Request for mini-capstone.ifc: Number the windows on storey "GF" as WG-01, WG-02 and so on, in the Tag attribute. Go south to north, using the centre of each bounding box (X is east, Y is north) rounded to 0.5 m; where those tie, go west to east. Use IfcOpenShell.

First a look at what the model holds.

```python
import ifcopenshell
import ifcopenshell.util.element
import ifcopenshell.util.placement

model = ifcopenshell.open("mini-capstone.ifc")
print(model.schema)
storey = next(s for s in model.by_type("IfcBuildingStorey") if s.Name == "GF")
windows = [e for e in ifcopenshell.util.element.get_decomposition(storey) if e.is_a("IfcWindow")]
for e in sorted(windows, key=lambda e: e.id()):
    origin = ifcopenshell.util.placement.get_local_placement(e.ObjectPlacement)[:3, 3]
    print(e.id(), e.Tag, e.Name, origin.round(2) + 0.0, sep=" | ")
```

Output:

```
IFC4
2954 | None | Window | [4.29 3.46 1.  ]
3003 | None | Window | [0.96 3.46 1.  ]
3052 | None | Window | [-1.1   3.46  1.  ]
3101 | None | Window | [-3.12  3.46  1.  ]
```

```python
import ifcopenshell
import ifcopenshell.geom
import ifcopenshell.util.element
import ifcopenshell.util.shape

model = ifcopenshell.open("mini-capstone.ifc")
settings = ifcopenshell.geom.settings()
settings.set("use-world-coords", True)


def centre(element):
    shape = ifcopenshell.geom.create_shape(settings, element)
    return ifcopenshell.util.shape.get_bbox_centroid(shape.geometry)


storey = next(s for s in model.by_type("IfcBuildingStorey") if s.Name == "GF")
windows = [e for e in ifcopenshell.util.element.get_decomposition(storey) if e.is_a("IfcWindow")]

# Insertion points can sit at a corner or the storey origin, so sort by the geometry (in metres).
centres = {e: centre(e) for e in windows}
windows.sort(key=lambda e: (round(centres[e][1] / 0.5), centres[e][0]))

for i, e in enumerate(windows, start=1):
    number = f"WG-{i:02d}"
    e.Tag = number
    print(e.id(), number)

model.write("mini-capstone_edited.ifc")
```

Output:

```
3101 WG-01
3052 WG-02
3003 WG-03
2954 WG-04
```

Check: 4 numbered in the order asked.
